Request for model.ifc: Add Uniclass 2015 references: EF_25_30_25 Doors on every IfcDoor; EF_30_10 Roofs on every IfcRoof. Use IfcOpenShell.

First a look at what the model holds.

```python
import ifcopenshell

model = ifcopenshell.open("model.ifc")
print(model.schema)
print("classifications:", [c.Name for c in model.by_type("IfcClassification")])
for ifc_class in ("IfcDoor", "IfcRoof", "IfcStair", "IfcWall", "IfcWindow"):
    print(ifc_class, len(model.by_type(ifc_class)))
```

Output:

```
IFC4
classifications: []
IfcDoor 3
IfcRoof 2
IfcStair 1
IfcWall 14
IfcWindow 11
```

```python
import ifcopenshell
import ifcopenshell.api.classification

model = ifcopenshell.open("model.ifc")

system = ifcopenshell.api.classification.add_classification(model, classification="Uniclass 2015")

codes = {
    "IfcDoor": ("EF_25_30_25", "Doors"),
    "IfcRoof": ("EF_30_10", "Roofs"),
}
for ifc_class, (code, name) in codes.items():
    products = model.by_type(ifc_class)
    ifcopenshell.api.classification.add_reference(
        model, products=products, classification=system, identification=code, name=name
    )
    print(code, len(products))

model.write("model_edited.ifc")
```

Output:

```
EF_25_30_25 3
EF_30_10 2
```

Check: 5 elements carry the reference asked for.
